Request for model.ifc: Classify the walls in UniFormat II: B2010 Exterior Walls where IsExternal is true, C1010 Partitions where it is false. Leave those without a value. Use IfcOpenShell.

First a look at what the model holds.

```python
import ifcopenshell
import ifcopenshell.util.element

model = ifcopenshell.open("model.ifc")
print(model.schema)
print("classifications:", [c.Name for c in model.by_type("IfcClassification")])
values = [ifcopenshell.util.element.get_pset(e, "Pset_WallCommon", "IsExternal") for e in model.by_type("IfcWall")]
for value in (True, False, None):
    print("IsExternal", value, values.count(value))
```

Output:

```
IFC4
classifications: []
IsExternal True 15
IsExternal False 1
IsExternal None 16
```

```python
import ifcopenshell
import ifcopenshell.api.classification
import ifcopenshell.util.element

model = ifcopenshell.open("model.ifc")

system = ifcopenshell.api.classification.add_classification(model, classification="UniFormat II")

walls = model.by_type("IfcWall")
external = {e: ifcopenshell.util.element.get_pset(e, "Pset_WallCommon", "IsExternal") for e in walls}
for flag, code, name in ((True, "B2010", "Exterior Walls"), (False, "C1010", "Partitions")):
    products = [e for e in walls if external[e] is flag]
    ifcopenshell.api.classification.add_reference(
        model, products=products, classification=system, identification=code, name=name
    )
    print(code, len(products))

model.write("model-out.ifc")
```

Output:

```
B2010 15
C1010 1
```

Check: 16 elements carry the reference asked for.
